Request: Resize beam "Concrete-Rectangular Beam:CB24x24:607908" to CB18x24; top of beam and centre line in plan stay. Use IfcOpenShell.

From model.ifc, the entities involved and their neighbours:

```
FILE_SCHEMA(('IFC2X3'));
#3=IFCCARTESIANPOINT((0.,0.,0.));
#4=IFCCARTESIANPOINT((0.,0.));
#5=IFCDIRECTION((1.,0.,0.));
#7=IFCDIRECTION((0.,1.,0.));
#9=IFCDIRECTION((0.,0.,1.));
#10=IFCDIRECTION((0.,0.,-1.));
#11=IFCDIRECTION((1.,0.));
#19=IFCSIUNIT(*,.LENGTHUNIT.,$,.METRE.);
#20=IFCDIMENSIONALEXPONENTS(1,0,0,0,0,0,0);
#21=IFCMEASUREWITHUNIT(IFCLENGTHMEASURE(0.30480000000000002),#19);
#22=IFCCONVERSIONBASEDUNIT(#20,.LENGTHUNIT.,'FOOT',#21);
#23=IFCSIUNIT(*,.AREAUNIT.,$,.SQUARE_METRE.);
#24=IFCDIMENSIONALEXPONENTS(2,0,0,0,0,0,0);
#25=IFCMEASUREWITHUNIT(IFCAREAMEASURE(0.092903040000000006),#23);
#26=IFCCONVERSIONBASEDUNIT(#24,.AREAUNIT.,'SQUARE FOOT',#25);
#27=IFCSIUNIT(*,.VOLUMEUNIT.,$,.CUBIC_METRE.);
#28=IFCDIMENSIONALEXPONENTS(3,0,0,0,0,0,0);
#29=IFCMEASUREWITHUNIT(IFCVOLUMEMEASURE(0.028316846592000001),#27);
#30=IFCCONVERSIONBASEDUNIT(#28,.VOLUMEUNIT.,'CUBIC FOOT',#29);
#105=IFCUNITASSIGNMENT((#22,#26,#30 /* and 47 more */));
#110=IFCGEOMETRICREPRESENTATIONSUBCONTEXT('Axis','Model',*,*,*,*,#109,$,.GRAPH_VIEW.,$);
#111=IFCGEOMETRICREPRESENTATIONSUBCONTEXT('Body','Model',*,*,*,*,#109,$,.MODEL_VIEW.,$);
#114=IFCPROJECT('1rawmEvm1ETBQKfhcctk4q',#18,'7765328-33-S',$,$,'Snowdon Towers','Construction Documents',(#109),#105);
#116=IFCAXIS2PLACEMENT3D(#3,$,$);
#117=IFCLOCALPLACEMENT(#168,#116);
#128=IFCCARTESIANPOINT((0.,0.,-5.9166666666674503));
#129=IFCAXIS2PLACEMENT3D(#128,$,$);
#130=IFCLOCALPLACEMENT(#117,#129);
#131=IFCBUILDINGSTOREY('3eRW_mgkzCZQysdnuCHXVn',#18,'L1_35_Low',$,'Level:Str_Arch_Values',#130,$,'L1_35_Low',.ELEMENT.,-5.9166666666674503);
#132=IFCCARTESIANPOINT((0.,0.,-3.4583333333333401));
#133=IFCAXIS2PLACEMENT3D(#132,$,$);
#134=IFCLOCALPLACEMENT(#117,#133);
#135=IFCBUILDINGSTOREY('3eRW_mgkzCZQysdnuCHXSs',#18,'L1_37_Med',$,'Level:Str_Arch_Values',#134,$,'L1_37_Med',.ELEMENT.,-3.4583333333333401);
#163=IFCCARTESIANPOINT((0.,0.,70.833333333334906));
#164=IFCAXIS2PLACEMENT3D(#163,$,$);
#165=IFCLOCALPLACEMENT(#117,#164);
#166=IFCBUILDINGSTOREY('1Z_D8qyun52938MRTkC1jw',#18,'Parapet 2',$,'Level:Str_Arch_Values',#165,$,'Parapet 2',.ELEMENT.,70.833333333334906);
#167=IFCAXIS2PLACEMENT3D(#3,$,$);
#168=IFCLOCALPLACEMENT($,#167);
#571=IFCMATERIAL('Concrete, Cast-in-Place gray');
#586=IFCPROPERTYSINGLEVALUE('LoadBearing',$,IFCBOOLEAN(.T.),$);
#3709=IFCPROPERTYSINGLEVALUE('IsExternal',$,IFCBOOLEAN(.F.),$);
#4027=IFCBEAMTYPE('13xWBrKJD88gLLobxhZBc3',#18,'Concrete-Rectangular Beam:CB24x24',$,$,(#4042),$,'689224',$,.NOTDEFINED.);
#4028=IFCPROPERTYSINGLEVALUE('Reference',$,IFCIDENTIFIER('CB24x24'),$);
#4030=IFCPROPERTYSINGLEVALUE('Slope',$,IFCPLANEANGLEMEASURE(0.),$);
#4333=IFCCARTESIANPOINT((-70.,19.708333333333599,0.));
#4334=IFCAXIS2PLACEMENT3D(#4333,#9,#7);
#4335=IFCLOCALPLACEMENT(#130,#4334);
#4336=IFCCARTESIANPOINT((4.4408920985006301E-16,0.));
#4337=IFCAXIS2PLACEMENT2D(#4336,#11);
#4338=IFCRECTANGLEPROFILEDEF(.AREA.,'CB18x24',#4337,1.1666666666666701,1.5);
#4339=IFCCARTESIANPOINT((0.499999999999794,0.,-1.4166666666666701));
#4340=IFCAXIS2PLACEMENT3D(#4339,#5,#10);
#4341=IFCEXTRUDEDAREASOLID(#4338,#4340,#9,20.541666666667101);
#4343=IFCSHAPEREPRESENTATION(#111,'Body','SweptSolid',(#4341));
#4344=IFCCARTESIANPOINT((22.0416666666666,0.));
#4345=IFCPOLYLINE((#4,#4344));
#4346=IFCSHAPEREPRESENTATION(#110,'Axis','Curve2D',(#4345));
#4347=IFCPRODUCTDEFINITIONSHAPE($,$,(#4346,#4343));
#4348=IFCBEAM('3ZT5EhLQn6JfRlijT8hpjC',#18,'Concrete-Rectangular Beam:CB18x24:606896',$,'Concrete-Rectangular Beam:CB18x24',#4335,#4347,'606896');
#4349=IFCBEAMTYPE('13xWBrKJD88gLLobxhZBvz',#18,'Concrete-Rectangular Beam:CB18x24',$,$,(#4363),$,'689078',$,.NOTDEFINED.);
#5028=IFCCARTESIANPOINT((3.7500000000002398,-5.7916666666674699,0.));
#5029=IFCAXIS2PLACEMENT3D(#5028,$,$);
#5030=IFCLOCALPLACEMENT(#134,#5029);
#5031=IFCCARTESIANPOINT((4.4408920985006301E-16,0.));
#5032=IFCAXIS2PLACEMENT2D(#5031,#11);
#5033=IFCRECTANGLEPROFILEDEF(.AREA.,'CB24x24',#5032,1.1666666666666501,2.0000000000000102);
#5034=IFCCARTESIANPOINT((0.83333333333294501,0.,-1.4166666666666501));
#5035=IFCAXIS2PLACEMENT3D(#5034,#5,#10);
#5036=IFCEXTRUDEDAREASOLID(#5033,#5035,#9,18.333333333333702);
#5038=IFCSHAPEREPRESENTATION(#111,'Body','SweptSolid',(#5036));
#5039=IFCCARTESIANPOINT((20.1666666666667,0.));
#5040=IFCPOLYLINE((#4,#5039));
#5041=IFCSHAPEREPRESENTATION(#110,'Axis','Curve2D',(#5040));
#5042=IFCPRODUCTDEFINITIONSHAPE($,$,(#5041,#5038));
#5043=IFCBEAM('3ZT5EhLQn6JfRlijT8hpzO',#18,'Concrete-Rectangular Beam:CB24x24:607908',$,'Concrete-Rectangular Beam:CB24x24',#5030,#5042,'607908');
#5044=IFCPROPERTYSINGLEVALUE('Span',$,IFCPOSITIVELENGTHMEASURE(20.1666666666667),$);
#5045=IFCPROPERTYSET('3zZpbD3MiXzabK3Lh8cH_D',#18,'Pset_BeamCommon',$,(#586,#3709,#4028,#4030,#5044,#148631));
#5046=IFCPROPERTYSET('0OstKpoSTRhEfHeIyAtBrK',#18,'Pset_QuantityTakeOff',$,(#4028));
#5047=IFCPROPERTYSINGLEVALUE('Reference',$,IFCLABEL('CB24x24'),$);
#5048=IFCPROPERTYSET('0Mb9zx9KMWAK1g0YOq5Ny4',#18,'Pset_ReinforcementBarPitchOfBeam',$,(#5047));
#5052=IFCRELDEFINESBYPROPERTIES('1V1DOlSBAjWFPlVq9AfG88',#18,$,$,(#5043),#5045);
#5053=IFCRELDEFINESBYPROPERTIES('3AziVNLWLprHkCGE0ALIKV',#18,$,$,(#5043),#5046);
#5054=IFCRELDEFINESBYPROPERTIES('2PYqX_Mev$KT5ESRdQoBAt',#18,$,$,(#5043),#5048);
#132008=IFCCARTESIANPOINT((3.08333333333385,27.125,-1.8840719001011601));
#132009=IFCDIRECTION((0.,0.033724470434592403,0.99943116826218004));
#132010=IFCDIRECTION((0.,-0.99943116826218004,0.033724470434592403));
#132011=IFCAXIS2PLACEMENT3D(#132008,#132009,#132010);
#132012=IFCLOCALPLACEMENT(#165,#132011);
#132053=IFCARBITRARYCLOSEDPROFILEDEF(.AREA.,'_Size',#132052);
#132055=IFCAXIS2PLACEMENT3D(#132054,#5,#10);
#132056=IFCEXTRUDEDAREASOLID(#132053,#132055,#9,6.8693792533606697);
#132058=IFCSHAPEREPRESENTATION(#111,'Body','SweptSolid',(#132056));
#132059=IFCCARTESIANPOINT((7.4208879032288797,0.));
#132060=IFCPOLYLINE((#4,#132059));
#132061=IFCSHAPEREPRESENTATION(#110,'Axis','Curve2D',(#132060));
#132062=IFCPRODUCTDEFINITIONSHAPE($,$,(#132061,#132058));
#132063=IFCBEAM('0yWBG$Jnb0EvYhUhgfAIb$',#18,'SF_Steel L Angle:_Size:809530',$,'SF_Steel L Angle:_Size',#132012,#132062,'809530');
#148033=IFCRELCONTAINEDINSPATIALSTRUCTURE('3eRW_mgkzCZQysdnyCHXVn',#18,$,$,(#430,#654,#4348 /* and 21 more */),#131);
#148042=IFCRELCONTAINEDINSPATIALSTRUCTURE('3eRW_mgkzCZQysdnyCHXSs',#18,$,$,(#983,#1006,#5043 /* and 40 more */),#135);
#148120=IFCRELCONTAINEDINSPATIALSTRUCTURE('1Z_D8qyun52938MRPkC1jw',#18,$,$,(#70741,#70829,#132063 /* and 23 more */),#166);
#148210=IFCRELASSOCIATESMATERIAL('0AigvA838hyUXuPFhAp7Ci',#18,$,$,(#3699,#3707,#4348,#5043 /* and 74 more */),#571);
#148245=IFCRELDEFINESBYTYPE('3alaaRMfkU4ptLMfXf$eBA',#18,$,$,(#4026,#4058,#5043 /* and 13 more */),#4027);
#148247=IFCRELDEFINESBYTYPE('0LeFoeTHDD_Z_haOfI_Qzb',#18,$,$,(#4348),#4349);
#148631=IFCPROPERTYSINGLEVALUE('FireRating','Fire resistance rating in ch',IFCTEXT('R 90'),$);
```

```python
import ifcopenshell
import ifcopenshell.api.pset
import ifcopenshell.api.type
import ifcopenshell.util.element
import ifcopenshell.util.representation

model = ifcopenshell.open("model.ifc")

member = model.by_guid("3ZT5EhLQn6JfRlijT8hpzO")
source = next(p for p in model.by_type("IfcRectangleProfileDef") if p.ProfileName == "CB18x24")

body = ifcopenshell.util.representation.get_representation(member, "Model", "Body")
solid = body.Items[0]
old_profile = solid.SweptArea

# Copy the section's sizes but keep this member's own profile position.
profile = ifcopenshell.util.element.copy(model, source)
# Profiles are centred, so shift by half the change in depth to hold the top.
shift = (old_profile.XDim - profile.XDim) / 2
x, y = old_profile.Position.Location.Coordinates
up = (-1.0, 0.0)  # upwards, in the solid's own plane
location = model.createIfcCartesianPoint((x + up[0] * shift, y + up[1] * shift))
profile.Position = model.createIfcAxis2Placement2D(location, old_profile.Position.RefDirection)
solid.SweptArea = profile
if not model.get_total_inverses(old_profile):
    ifcopenshell.util.element.remove_deep2(model, old_profile)

new_type = model.by_guid("13xWBrKJD88gLLobxhZBvz")
ifcopenshell.api.type.assign_type(
    model, related_objects=[member], relating_type=new_type, should_map_representations=False
)
member.Name = member.Name.replace("CB24x24", "CB18x24")
member.ObjectType = "Concrete-Rectangular Beam:CB18x24"
pset = model.by_id(ifcopenshell.util.element.get_pset(member, "Pset_BeamCommon", should_inherit=False)["id"])
ifcopenshell.api.pset.edit_pset(model, pset=pset, properties={"Reference": "CB18x24"})
pset = model.by_id(ifcopenshell.util.element.get_pset(member, "Pset_QuantityTakeOff", should_inherit=False)["id"])
ifcopenshell.api.pset.edit_pset(model, pset=pset, properties={"Reference": "CB18x24"})
pset = model.by_id(ifcopenshell.util.element.get_pset(member, "Pset_ReinforcementBarPitchOfBeam", should_inherit=False)["id"])
ifcopenshell.api.pset.edit_pset(model, pset=pset, properties={"Reference": "CB18x24"})

print(solid.SweptArea)

model.write("model_v2.ifc")
```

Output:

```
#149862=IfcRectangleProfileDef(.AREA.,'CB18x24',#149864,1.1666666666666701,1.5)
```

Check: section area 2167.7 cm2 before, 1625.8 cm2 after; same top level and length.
